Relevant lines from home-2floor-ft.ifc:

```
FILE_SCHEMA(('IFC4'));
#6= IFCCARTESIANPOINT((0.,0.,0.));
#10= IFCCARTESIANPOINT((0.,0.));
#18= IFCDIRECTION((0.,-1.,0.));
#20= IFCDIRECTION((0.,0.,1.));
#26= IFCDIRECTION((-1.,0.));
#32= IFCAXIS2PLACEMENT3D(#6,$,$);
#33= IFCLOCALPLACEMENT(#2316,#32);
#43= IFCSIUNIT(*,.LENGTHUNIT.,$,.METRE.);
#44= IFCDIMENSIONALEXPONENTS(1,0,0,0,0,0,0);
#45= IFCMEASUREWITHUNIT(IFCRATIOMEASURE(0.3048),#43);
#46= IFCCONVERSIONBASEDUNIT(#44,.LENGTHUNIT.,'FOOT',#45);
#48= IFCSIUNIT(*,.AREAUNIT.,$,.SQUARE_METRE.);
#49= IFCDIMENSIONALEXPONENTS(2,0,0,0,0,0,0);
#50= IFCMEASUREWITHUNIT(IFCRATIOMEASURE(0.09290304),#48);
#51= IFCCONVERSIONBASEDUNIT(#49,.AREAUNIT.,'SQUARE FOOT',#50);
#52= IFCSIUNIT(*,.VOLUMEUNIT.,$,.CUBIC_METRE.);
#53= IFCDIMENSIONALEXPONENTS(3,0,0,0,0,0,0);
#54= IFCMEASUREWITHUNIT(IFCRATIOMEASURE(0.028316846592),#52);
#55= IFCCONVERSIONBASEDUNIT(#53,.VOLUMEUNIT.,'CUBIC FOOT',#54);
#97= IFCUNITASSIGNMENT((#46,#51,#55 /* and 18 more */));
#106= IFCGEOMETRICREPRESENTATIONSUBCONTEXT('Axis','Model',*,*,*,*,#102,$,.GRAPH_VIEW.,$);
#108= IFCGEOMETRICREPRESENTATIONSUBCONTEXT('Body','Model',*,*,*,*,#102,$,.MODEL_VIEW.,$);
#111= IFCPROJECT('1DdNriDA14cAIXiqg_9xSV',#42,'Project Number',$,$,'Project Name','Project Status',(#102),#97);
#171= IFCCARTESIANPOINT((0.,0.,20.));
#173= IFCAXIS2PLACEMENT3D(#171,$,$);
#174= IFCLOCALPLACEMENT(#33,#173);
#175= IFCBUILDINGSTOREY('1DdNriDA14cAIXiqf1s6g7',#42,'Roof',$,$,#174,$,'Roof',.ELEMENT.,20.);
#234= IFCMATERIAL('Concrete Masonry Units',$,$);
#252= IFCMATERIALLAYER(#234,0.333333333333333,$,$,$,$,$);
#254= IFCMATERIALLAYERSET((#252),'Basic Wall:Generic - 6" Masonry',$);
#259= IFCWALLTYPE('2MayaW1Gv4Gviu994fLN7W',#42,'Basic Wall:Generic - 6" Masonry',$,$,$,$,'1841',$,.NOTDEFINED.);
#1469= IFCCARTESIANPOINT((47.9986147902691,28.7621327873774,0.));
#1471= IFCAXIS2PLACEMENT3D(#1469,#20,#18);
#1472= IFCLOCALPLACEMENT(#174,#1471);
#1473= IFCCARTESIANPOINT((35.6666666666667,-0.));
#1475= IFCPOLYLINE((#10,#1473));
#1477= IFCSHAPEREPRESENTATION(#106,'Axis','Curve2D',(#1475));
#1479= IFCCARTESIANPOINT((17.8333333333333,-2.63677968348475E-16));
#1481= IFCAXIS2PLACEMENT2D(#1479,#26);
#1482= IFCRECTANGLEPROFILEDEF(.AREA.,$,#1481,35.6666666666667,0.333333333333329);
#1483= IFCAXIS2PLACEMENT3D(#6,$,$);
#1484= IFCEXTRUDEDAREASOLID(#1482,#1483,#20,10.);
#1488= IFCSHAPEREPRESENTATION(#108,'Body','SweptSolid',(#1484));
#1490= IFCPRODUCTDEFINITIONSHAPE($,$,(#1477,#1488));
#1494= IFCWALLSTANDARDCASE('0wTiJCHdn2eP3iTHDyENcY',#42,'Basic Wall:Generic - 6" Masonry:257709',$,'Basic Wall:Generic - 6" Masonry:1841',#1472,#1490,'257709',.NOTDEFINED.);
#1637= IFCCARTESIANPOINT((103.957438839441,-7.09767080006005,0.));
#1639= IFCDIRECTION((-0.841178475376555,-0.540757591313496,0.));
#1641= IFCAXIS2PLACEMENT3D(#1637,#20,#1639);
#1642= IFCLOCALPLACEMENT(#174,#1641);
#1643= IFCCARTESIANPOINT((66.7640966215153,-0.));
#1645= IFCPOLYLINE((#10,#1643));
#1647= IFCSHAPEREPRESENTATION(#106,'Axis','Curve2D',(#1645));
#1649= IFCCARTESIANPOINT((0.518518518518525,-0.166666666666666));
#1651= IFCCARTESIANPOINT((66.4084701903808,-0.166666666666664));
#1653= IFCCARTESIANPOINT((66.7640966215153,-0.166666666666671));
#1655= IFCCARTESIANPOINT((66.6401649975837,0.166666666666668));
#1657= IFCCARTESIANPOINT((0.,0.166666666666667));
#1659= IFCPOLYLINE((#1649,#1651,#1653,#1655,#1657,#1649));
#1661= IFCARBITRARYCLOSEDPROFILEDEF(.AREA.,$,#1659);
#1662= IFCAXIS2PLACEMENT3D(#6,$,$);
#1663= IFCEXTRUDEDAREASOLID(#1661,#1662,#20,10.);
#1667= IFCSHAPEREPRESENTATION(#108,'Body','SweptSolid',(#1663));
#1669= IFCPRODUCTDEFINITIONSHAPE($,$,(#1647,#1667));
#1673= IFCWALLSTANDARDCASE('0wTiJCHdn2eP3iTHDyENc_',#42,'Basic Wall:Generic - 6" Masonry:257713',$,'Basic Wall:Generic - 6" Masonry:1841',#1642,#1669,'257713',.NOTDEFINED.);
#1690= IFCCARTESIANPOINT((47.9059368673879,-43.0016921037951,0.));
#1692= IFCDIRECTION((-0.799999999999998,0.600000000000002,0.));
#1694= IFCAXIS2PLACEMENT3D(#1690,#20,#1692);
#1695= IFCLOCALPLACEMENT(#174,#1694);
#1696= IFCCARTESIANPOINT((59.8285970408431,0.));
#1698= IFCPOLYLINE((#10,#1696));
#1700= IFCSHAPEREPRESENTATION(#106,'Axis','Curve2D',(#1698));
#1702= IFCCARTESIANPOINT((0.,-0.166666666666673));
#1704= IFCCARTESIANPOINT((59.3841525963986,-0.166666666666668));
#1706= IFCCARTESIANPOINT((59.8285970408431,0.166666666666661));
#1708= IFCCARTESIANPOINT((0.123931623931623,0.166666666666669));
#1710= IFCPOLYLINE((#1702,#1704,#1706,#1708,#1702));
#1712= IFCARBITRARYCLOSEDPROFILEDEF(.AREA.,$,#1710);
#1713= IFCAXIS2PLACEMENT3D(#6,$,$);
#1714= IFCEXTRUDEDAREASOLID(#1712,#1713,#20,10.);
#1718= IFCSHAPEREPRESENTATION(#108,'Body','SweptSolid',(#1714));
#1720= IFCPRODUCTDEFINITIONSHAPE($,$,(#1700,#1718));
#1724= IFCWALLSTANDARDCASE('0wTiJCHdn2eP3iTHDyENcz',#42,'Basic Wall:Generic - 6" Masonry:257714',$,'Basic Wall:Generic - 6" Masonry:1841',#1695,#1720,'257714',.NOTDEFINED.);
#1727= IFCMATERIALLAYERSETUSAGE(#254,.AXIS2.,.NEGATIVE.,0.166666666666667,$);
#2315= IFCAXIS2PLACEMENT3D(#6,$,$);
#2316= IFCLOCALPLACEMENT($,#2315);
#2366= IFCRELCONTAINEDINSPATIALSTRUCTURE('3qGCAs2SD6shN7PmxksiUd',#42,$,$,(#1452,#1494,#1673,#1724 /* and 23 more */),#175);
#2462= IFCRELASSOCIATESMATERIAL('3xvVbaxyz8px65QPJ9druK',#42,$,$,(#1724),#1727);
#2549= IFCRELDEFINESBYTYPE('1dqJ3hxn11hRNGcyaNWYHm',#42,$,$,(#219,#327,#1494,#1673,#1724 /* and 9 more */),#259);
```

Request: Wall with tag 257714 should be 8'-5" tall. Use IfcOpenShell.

```python
import ifcopenshell
import ifcopenshell.geom
import ifcopenshell.util.representation
import ifcopenshell.util.shape
import ifcopenshell.util.unit

model = ifcopenshell.open("home-2floor-ft.ifc")
unit_scale = ifcopenshell.util.unit.calculate_unit_scale(model)
settings = ifcopenshell.geom.settings()


def volume(element):
    """Net volume in cubic metres, openings subtracted."""
    shape = ifcopenshell.geom.create_shape(settings, element)
    return ifcopenshell.util.shape.get_volume(shape.geometry)


wall = model.by_guid("0wTiJCHdn2eP3iTHDyENcz")
before = volume(wall)

body = ifcopenshell.util.representation.get_representation(wall, "Model", "Body")
solid = body.Items[0]
old_height = solid.Depth
solid.Depth = 101 * 0.0254 / unit_scale
after = volume(wall)

print(f"height {old_height:g} -> {solid.Depth:g}, volume {before:.3f} -> {after:.3f} m3")

model.write("home-2floor-ft_v2.ifc")
```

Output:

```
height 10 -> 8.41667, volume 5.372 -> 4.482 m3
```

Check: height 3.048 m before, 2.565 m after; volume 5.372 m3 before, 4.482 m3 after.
